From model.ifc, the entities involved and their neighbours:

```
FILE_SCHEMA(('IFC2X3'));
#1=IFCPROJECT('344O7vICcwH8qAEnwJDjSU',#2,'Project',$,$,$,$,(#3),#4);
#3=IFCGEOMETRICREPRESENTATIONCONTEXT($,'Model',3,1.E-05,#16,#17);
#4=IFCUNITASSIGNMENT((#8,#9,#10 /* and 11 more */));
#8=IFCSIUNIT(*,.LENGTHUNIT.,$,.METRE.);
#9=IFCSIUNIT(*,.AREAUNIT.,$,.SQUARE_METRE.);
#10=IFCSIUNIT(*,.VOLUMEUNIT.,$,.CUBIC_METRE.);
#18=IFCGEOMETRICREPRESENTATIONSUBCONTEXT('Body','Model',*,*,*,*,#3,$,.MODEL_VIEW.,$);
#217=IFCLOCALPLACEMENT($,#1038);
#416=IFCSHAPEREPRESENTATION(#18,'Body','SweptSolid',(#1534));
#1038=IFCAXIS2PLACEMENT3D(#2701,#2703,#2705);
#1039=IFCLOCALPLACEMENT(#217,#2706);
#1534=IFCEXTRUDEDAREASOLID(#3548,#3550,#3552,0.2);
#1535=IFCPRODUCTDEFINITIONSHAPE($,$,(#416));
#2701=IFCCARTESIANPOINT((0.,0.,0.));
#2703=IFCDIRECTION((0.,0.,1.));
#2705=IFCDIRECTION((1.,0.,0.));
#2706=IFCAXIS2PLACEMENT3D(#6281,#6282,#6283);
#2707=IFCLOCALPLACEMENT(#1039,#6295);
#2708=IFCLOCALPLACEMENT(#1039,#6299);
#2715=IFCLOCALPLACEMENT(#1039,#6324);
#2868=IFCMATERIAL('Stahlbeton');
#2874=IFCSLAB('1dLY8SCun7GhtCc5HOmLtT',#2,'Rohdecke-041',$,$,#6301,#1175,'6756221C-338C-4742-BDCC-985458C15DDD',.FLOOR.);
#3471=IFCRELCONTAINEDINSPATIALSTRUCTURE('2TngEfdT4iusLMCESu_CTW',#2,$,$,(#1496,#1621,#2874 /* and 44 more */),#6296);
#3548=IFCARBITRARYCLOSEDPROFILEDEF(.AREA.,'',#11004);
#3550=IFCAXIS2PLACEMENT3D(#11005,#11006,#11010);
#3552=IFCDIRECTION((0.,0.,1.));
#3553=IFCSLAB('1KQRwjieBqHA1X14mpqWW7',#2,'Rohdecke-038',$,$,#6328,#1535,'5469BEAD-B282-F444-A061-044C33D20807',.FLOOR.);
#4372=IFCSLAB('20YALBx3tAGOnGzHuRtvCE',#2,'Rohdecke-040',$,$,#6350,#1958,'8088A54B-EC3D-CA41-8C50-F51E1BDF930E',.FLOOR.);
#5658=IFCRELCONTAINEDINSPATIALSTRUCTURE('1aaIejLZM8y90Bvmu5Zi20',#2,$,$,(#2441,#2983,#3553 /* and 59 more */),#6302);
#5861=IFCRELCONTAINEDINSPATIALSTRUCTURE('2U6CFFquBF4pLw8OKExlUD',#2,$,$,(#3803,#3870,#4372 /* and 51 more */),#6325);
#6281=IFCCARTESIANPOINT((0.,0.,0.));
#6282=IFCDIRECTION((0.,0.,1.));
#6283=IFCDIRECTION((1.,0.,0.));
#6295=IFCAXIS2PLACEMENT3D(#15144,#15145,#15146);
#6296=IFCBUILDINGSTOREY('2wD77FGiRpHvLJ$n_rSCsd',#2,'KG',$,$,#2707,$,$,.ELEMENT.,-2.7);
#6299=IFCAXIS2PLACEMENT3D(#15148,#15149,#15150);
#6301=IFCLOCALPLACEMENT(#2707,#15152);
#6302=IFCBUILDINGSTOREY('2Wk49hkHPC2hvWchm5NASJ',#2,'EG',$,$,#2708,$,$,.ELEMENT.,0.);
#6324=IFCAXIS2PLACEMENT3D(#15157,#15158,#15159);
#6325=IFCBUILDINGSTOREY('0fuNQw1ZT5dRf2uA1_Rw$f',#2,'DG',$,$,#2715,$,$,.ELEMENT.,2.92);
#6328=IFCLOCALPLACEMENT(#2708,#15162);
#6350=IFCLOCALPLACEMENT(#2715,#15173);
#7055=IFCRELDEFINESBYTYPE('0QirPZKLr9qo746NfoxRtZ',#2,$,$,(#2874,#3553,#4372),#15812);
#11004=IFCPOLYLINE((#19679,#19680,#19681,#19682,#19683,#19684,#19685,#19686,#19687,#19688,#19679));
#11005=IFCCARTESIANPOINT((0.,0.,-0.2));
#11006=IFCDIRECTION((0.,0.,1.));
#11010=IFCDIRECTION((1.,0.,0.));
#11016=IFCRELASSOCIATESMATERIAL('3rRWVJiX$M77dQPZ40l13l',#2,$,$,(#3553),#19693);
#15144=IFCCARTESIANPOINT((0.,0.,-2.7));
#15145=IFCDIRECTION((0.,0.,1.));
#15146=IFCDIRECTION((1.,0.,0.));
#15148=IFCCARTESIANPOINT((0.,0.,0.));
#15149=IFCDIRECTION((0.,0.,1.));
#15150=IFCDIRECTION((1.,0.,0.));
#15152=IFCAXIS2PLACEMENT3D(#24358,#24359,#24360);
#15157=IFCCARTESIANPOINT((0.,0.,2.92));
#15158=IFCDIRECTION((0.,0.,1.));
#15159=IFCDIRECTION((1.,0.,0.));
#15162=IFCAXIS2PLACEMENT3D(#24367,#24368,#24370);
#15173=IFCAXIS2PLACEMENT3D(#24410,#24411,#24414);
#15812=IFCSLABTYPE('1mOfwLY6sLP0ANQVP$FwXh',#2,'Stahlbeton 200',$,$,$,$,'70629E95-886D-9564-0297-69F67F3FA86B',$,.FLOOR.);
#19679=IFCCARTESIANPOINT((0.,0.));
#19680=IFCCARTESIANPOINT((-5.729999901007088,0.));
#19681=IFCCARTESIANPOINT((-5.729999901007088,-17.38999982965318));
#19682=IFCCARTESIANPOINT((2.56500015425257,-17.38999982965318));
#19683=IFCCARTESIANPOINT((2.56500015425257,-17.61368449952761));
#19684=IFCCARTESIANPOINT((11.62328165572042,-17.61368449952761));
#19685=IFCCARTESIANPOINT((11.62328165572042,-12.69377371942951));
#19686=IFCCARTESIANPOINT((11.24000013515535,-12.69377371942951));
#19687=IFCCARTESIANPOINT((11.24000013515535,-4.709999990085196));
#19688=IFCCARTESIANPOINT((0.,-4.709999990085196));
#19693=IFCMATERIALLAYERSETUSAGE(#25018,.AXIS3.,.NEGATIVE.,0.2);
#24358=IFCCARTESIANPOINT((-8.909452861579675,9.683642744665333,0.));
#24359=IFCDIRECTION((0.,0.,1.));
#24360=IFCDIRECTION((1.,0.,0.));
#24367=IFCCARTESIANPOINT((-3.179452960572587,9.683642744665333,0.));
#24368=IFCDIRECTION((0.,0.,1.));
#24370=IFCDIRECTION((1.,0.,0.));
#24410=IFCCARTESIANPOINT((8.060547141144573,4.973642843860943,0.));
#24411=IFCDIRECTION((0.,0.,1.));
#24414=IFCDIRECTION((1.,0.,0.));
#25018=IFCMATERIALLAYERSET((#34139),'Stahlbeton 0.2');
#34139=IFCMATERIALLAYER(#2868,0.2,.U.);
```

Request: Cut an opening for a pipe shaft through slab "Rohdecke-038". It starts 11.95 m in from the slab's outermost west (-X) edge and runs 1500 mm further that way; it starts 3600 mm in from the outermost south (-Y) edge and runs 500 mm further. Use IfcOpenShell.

```python
import numpy as np
import ifcopenshell
import ifcopenshell.api.feature
import ifcopenshell.api.geometry
import ifcopenshell.api.root
import ifcopenshell.geom
import ifcopenshell.util.placement
import ifcopenshell.util.representation
import ifcopenshell.util.shape
import ifcopenshell.util.unit

model = ifcopenshell.open("model.ifc")
unit_scale = ifcopenshell.util.unit.calculate_unit_scale(model)
settings = ifcopenshell.geom.settings()


def volume(element):
    """Net volume in cubic metres, openings subtracted."""
    shape = ifcopenshell.geom.create_shape(settings, element)
    return ifcopenshell.util.shape.get_volume(shape.geometry)


slab = model.by_id(3553)
before = volume(slab)

# Extent in the slab's own axes, in metres. The edges named are its -X and -Y sides.
slab_shape = ifcopenshell.geom.create_shape(settings, slab)
vertices = ifcopenshell.util.shape.get_vertices(slab_shape.geometry)
x_min, y_min, bottom = vertices.min(axis=0)
top = vertices[:, 2].max()

opening = ifcopenshell.api.root.create_entity(model, ifc_class="IfcOpeningElement", name="Pipe shaft opening")
context = ifcopenshell.util.representation.get_context(model, "Model", "Body", "MODEL_VIEW")
width, depth = 1.5, 0.5
outline = [(0.0, 0.0), (width, 0.0), (width, depth), (0.0, depth), (0.0, 0.0)]
# Overshoot both faces by 50 mm so the cut is clean.
shape = ifcopenshell.api.geometry.add_slab_representation(
    model, context=context, depth=top - bottom + 0.1, polyline=outline
)
ifcopenshell.api.geometry.assign_representation(model, product=opening, representation=shape)

matrix = ifcopenshell.util.placement.get_local_placement(slab.ObjectPlacement)
matrix[:, 3] = matrix @ np.append(np.array([x_min + 11.95, y_min + 3.6, bottom - 0.05]) / unit_scale, 1.0)
ifcopenshell.api.geometry.edit_object_placement(model, product=opening, matrix=matrix, is_si=False)
ifcopenshell.api.feature.add_feature(model, feature=opening, element=slab)

after = volume(slab)

print(f"slab volume {before:.3f} -> {after:.3f} m3")

model.write("model_v2.ifc")
```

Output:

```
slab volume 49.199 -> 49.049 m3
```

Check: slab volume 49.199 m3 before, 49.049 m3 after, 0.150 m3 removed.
